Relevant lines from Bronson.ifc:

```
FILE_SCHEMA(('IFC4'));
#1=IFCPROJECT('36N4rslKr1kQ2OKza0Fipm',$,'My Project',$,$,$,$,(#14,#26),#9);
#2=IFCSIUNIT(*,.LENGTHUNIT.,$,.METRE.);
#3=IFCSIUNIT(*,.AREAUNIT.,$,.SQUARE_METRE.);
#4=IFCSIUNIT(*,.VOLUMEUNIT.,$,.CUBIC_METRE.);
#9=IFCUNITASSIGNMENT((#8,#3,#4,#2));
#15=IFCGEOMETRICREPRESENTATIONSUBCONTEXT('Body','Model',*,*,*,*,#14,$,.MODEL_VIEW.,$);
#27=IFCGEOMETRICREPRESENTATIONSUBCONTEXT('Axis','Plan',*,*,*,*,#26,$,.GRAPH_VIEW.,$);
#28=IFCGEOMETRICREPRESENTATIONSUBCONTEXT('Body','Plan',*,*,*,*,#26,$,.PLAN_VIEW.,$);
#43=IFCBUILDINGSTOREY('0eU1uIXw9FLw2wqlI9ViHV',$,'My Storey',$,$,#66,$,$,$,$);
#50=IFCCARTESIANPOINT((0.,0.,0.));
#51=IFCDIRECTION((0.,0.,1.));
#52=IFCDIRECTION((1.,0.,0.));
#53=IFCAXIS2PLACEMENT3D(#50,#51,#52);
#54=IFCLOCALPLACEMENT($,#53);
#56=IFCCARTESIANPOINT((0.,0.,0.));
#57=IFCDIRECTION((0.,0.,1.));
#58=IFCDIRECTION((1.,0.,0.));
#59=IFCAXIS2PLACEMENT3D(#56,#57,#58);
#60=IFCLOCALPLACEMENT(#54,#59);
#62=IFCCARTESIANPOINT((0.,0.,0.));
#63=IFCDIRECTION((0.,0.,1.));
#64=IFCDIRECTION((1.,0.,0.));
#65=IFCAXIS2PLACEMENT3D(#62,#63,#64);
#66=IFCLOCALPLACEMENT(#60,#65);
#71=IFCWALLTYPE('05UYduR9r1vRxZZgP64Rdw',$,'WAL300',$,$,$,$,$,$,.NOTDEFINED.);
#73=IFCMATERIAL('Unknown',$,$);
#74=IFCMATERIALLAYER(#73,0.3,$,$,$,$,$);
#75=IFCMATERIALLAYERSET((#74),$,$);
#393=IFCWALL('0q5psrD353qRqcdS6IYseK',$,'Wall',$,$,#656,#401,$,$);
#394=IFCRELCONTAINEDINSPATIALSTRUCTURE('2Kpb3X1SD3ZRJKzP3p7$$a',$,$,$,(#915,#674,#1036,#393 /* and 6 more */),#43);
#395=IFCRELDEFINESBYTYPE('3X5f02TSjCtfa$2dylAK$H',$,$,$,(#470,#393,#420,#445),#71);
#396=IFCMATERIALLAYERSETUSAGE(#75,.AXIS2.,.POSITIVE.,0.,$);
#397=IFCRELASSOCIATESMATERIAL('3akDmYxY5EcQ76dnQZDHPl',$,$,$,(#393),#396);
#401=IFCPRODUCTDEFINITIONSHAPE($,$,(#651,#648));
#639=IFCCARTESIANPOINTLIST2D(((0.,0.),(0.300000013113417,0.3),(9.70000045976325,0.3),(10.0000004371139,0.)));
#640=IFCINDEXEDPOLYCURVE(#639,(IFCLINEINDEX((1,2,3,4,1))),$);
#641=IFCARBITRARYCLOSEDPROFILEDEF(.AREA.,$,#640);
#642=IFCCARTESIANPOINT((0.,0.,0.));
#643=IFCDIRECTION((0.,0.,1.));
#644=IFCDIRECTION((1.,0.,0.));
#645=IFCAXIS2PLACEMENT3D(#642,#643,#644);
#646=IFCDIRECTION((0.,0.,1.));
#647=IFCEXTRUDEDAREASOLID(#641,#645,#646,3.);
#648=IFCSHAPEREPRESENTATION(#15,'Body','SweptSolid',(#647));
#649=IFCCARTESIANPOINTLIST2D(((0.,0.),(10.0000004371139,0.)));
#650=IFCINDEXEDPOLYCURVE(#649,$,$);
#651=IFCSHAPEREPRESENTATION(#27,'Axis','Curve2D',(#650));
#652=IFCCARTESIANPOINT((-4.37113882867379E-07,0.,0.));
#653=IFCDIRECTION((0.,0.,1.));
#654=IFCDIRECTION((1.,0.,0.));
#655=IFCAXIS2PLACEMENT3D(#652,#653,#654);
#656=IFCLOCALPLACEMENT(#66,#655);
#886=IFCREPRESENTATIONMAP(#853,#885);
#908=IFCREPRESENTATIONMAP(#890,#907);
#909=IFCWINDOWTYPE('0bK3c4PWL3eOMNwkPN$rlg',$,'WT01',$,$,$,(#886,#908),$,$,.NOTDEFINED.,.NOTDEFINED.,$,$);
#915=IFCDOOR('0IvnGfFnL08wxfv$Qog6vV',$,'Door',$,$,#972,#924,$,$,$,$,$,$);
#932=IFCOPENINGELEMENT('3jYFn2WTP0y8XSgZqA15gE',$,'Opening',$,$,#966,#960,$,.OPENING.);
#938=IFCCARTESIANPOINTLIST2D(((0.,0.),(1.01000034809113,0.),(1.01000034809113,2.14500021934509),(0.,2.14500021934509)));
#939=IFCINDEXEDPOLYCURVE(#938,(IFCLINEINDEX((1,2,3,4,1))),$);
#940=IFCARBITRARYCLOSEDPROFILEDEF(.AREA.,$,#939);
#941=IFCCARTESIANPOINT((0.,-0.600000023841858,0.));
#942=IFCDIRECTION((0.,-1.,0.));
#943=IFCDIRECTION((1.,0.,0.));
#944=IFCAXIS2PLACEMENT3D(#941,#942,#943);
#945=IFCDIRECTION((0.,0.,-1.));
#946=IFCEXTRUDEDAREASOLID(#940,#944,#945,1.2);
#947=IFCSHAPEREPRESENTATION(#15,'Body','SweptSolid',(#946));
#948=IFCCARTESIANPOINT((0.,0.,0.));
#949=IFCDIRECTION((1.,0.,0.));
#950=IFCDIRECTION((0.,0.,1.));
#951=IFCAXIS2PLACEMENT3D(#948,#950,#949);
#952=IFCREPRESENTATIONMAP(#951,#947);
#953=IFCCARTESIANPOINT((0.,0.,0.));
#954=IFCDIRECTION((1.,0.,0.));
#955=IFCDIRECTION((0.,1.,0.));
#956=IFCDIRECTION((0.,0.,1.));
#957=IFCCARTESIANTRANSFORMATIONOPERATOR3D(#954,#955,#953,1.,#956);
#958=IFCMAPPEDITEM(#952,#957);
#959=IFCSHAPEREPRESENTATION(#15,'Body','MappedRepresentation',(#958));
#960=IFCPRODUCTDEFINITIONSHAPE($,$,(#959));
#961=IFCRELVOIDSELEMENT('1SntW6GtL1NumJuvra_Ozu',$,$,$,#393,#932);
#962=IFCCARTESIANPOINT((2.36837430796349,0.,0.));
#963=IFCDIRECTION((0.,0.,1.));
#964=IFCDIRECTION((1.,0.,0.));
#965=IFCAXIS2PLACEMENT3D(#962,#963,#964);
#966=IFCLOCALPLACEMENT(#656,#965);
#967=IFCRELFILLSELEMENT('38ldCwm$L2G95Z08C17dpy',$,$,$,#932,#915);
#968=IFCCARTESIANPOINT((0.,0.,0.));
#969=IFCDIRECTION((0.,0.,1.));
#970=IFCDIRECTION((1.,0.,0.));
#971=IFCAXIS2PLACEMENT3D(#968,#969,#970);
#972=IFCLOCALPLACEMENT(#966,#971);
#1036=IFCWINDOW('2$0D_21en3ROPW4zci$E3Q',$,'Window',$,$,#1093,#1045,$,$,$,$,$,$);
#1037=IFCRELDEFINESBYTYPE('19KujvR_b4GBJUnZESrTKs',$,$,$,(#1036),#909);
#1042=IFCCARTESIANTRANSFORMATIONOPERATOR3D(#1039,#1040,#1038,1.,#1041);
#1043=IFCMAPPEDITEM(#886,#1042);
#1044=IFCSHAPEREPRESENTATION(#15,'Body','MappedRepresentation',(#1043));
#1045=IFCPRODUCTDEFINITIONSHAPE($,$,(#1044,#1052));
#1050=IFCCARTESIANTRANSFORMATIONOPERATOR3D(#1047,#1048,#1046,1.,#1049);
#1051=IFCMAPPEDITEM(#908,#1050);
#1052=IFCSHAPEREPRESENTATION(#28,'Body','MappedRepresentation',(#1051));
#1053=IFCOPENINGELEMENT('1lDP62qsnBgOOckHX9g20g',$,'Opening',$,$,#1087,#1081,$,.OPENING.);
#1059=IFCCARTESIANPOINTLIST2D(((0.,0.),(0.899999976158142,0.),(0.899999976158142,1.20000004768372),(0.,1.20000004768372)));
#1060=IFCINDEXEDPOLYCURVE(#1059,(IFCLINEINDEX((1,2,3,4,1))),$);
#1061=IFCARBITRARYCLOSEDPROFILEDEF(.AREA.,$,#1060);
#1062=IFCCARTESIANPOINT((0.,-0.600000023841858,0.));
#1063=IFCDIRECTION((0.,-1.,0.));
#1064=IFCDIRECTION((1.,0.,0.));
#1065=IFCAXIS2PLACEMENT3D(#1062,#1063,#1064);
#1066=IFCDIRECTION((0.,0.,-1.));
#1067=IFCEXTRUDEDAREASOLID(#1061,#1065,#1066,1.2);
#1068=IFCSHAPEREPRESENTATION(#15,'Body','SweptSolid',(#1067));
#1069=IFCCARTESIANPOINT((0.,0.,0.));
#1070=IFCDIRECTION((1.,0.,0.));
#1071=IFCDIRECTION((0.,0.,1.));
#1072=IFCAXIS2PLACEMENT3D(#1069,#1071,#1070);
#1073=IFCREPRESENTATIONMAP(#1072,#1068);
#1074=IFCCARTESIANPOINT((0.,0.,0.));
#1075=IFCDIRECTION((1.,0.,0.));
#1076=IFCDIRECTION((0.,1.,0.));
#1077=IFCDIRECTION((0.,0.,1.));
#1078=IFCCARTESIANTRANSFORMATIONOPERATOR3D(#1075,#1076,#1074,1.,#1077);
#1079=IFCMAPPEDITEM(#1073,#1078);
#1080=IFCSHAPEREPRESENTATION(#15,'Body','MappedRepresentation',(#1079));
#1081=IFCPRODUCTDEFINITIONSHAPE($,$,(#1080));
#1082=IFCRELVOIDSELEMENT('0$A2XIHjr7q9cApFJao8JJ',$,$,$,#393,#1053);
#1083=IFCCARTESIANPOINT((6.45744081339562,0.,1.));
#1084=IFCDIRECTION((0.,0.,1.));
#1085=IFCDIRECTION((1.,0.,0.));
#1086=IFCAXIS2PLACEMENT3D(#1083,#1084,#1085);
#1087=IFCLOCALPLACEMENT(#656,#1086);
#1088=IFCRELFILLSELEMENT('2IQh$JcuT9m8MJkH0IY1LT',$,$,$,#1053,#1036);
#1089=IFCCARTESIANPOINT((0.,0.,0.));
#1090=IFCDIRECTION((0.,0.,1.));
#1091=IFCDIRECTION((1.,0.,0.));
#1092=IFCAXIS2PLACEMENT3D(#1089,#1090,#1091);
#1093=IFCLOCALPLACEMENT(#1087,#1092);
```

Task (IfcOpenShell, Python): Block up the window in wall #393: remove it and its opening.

```python
import ifcopenshell
import ifcopenshell.api.feature
import ifcopenshell.api.root
import ifcopenshell.geom
import ifcopenshell.util.shape

model = ifcopenshell.open("Bronson.ifc")
settings = ifcopenshell.geom.settings()


def volume(element):
    """Net volume in cubic metres, openings subtracted."""
    shape = ifcopenshell.geom.create_shape(settings, element)
    return ifcopenshell.util.shape.get_volume(shape.geometry)


window = model.by_id(1036)
opening = window.FillsVoids[0].RelatingOpeningElement
wall = opening.VoidsElements[0].RelatingBuildingElement
before = volume(wall)

ifcopenshell.api.root.remove_product(model, product=window)
ifcopenshell.api.feature.remove_feature(model, feature=opening)

after = volume(wall)

print(f"wall volume {before:.3f} -> {after:.3f} m3")

model.write("Bronson_edited.ifc")
```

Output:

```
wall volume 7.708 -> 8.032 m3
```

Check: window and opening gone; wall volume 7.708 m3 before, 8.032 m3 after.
